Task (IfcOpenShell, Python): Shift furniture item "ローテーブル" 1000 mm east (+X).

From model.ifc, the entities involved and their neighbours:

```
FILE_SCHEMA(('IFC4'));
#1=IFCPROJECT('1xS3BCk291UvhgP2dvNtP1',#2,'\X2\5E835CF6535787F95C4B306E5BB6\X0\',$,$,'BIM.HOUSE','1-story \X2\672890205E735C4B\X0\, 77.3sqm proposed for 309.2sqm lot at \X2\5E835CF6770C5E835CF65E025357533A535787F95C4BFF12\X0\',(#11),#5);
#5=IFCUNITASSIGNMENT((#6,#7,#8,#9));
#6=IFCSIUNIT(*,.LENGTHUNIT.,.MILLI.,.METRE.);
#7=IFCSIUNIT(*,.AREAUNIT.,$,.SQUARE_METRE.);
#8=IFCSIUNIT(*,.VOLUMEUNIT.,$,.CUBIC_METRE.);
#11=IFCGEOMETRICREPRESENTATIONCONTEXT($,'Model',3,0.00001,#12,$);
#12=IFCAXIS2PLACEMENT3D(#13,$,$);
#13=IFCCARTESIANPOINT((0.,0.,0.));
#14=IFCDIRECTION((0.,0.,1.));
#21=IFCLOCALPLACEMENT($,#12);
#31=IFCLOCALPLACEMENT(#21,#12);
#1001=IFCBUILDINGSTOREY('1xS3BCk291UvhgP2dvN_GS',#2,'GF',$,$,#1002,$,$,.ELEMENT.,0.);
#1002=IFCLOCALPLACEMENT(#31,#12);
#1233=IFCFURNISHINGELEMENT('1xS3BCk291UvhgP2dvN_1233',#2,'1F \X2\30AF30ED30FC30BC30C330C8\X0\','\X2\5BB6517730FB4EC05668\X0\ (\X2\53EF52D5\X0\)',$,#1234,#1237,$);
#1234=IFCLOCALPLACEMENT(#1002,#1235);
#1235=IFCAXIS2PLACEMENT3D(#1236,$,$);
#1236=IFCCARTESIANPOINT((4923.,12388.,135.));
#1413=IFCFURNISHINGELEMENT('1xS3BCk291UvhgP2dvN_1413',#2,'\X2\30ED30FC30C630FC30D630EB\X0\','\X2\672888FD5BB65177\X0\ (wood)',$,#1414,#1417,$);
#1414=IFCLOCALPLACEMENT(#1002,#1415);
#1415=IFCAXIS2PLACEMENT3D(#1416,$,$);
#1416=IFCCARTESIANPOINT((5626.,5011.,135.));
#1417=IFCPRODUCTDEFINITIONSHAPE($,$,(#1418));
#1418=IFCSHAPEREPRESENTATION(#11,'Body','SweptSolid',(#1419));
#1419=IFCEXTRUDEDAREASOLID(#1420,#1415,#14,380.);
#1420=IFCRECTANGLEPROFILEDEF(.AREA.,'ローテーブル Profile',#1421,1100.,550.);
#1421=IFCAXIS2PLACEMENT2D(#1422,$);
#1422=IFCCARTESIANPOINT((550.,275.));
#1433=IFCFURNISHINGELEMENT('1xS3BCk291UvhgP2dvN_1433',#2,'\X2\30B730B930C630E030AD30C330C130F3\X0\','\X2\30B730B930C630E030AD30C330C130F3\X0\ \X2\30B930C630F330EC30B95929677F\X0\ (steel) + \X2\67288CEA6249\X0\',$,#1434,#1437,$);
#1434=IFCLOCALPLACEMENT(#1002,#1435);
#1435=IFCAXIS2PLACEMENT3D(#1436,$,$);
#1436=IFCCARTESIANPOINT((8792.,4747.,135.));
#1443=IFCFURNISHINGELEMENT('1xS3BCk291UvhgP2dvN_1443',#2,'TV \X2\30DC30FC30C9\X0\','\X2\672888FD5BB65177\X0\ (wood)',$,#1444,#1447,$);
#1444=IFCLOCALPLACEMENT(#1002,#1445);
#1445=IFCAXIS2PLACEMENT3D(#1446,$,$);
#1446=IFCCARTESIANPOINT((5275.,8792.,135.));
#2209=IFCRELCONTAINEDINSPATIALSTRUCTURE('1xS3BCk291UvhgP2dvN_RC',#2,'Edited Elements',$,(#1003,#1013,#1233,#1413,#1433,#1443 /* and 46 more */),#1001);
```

```python
import ifcopenshell
import ifcopenshell.api.geometry
import ifcopenshell.util.placement
import ifcopenshell.util.unit

model = ifcopenshell.open("model.ifc")
unit_scale = ifcopenshell.util.unit.calculate_unit_scale(model)

item = model.by_guid("1xS3BCk291UvhgP2dvN_1413")
matrix = ifcopenshell.util.placement.get_local_placement(item.ObjectPlacement)
matrix[0, 3] += 1 / unit_scale
ifcopenshell.api.geometry.edit_object_placement(model, product=item, matrix=matrix, is_si=False)

print(ifcopenshell.util.placement.get_local_placement(item.ObjectPlacement).round(3) + 0.0)

model.write("model_v2.ifc")
```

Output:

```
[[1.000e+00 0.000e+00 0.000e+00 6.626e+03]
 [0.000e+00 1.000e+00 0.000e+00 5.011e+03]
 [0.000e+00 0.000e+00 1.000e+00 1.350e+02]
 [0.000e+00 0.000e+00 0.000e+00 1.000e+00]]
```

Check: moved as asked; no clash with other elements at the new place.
